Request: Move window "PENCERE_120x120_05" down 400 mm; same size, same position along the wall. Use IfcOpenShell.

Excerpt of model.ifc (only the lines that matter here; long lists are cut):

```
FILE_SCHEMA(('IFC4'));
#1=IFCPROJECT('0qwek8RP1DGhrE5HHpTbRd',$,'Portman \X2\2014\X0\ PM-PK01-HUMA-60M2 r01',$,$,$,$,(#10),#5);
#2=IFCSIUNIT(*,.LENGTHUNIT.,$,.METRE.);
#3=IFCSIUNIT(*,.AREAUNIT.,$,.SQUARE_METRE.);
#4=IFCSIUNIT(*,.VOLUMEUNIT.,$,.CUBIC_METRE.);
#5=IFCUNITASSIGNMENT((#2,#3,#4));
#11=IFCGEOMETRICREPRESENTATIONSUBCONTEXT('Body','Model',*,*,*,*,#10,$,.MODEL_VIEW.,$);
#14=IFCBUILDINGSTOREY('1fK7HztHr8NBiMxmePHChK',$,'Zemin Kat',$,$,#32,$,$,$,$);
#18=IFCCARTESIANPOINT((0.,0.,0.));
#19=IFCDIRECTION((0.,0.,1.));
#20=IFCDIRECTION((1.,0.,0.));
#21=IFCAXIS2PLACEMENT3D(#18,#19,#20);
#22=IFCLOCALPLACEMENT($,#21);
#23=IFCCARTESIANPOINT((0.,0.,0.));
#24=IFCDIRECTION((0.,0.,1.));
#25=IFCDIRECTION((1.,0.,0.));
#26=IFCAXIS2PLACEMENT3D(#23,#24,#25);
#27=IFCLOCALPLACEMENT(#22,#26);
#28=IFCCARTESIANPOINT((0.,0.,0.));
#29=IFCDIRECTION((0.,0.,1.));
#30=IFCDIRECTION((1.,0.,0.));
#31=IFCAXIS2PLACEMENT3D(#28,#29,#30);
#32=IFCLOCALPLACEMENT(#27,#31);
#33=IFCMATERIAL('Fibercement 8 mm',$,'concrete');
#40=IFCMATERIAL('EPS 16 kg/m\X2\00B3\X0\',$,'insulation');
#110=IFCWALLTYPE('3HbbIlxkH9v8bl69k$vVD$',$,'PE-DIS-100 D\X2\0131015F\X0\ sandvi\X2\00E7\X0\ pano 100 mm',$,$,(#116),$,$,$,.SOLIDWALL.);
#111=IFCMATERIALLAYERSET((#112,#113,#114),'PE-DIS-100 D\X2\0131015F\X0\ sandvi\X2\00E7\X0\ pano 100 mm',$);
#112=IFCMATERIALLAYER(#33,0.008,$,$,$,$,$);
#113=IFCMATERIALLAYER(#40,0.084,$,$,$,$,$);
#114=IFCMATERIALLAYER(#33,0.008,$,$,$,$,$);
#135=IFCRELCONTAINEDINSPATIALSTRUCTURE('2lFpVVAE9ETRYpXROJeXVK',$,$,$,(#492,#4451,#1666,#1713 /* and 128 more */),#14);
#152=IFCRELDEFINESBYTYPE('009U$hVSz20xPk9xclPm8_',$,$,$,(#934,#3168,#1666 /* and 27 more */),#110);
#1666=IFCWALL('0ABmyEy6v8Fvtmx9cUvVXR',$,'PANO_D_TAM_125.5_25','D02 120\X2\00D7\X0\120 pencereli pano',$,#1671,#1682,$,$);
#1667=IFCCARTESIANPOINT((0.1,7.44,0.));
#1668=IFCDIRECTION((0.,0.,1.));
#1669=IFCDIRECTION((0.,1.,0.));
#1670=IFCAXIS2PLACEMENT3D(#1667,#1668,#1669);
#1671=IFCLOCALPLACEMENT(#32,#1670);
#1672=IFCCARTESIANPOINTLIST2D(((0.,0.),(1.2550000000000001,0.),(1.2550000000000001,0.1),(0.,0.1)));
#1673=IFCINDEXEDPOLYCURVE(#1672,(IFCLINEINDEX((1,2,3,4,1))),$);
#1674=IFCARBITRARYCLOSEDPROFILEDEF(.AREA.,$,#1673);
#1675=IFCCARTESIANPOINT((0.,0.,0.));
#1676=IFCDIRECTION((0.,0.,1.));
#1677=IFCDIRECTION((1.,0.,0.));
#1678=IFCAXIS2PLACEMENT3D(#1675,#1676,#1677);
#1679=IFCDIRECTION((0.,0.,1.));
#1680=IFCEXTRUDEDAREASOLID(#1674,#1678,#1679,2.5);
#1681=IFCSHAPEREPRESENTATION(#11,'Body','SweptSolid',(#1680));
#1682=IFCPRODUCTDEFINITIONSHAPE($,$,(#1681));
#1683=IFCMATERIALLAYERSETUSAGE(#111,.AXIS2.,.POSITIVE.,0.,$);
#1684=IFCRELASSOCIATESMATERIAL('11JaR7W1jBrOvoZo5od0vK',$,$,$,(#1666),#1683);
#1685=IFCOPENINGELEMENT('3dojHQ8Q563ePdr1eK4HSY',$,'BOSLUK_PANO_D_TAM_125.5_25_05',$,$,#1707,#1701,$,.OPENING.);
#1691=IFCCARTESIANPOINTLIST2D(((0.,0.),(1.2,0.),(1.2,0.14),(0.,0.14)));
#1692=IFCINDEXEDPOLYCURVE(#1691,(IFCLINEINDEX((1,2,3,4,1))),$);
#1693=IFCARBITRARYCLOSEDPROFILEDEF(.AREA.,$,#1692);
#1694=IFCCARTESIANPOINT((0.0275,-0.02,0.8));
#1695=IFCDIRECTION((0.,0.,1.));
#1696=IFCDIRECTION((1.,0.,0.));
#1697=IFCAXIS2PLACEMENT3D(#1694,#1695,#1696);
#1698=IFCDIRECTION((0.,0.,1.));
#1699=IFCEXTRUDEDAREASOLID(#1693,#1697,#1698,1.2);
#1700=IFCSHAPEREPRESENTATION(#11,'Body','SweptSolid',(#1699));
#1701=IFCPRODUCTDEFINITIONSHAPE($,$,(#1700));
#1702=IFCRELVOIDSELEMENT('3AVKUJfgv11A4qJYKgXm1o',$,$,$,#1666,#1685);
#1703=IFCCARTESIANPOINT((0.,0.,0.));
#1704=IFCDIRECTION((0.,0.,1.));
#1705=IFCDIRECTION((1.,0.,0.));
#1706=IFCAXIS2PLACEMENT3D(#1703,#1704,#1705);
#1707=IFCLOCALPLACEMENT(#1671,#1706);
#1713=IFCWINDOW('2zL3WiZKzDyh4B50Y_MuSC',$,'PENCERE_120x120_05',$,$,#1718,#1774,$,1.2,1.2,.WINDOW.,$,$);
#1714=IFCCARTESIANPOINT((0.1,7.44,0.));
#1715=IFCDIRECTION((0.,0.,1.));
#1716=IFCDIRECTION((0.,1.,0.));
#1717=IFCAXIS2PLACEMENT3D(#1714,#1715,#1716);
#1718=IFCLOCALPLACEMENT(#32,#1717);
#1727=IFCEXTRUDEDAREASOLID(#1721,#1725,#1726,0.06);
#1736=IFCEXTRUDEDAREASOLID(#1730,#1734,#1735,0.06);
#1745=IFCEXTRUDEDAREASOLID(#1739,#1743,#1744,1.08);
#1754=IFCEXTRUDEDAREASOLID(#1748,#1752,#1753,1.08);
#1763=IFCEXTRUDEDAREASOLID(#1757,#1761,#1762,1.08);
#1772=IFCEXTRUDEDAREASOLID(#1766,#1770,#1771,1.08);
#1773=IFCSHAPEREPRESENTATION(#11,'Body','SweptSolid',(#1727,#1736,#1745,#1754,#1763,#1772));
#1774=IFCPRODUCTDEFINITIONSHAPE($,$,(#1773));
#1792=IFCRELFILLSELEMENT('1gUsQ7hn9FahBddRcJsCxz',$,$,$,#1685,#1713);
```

```python
import numpy as np
import ifcopenshell
import ifcopenshell.api.geometry
import ifcopenshell.util.placement
import ifcopenshell.util.unit

model = ifcopenshell.open("model.ifc")
unit_scale = ifcopenshell.util.unit.calculate_unit_scale(model)

window = model.by_guid("2zL3WiZKzDyh4B50Y_MuSC")
opening = window.FillsVoids[0].RelatingOpeningElement
dz = -0.4

shift = np.array([0.0, 0.0, dz])
# The window is not placed relative to its opening, so move both.
for product in (opening, window):
    matrix = ifcopenshell.util.placement.get_local_placement(product.ObjectPlacement)
    matrix[:3, 3] += shift
    ifcopenshell.api.geometry.edit_object_placement(model, product=product, matrix=matrix, is_si=False)

print(f"moved by {dz * unit_scale:+.3f} m")

model.write("model_edited.ifc")
```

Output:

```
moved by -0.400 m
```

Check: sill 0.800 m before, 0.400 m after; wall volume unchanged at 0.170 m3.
